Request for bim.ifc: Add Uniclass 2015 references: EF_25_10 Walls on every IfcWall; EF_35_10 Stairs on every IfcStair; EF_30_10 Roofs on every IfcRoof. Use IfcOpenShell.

First a look at what the model holds.

```python
import ifcopenshell

model = ifcopenshell.open("bim.ifc")
print(model.schema)
print("classifications:", [c.Name for c in model.by_type("IfcClassification")])
for ifc_class in ("IfcDoor", "IfcRoof", "IfcStair", "IfcWall", "IfcWindow"):
    print(ifc_class, len(model.by_type(ifc_class)))
```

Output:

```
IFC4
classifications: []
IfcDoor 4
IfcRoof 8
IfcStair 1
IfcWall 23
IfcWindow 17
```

```python
import ifcopenshell
import ifcopenshell.api.classification

model = ifcopenshell.open("bim.ifc")

system = ifcopenshell.api.classification.add_classification(model, classification="Uniclass 2015")

codes = {
    "IfcWall": ("EF_25_10", "Walls"),
    "IfcStair": ("EF_35_10", "Stairs"),
    "IfcRoof": ("EF_30_10", "Roofs"),
}
for ifc_class, (code, name) in codes.items():
    products = model.by_type(ifc_class)
    ifcopenshell.api.classification.add_reference(
        model, products=products, classification=system, identification=code, name=name
    )
    print(code, len(products))

model.write("bim_updated.ifc")
```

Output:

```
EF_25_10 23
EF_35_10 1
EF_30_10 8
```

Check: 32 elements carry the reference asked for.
